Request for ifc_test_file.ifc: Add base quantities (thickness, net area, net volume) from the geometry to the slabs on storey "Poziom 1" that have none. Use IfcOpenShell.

First a look at what the model holds.

```python
import ifcopenshell
import ifcopenshell.util.element
import ifcopenshell.util.unit

model = ifcopenshell.open("ifc_test_file.ifc")
print(model.schema)
for unit_type in ("LENGTHUNIT", "AREAUNIT", "VOLUMEUNIT"):
    print(unit_type, ifcopenshell.util.unit.calculate_unit_scale(model, unit_type))
storey = next(s for s in model.by_type("IfcBuildingStorey") if s.Name == "Poziom 1")
slabs = [e for e in ifcopenshell.util.element.get_decomposition(storey) if e.is_a("IfcSlab")]
for e in sorted(slabs, key=lambda e: e.id()):
    print(e.id(), e.is_a(), e.Name, list(ifcopenshell.util.element.get_psets(e, qtos_only=True)), sep=" | ")
```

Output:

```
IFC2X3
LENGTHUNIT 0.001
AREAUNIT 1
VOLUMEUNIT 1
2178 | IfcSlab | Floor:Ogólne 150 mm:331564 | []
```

```python
import ifcopenshell
import ifcopenshell.api.pset
import ifcopenshell.geom
import ifcopenshell.util.element
import ifcopenshell.util.shape
import ifcopenshell.util.unit

model = ifcopenshell.open("ifc_test_file.ifc")
unit_scale = ifcopenshell.util.unit.calculate_unit_scale(model)
area_scale = ifcopenshell.util.unit.calculate_unit_scale(model, "AREAUNIT")
volume_scale = ifcopenshell.util.unit.calculate_unit_scale(model, "VOLUMEUNIT")
settings = ifcopenshell.geom.settings()

storey = next(s for s in model.by_type("IfcBuildingStorey") if s.Name == "Poziom 1")
slabs = [e for e in ifcopenshell.util.element.get_decomposition(storey) if e.is_a("IfcSlab")]

for e in sorted(slabs, key=lambda e: e.id()):
    if ifcopenshell.util.element.get_psets(e, qtos_only=True, should_inherit=False):
        continue
    # Geometry comes back in metres, in the element's own axes.
    shape = ifcopenshell.geom.create_shape(settings, e)
    values = {
        "Width": ifcopenshell.util.shape.get_z(shape.geometry) / unit_scale,
        "NetArea": ifcopenshell.util.shape.get_footprint_area(shape.geometry) / area_scale,
        "NetVolume": ifcopenshell.util.shape.get_volume(shape.geometry) / volume_scale,
    }
    qto = ifcopenshell.api.pset.add_qto(model, product=e, name="BaseQuantities")
    ifcopenshell.api.pset.edit_qto(model, qto=qto, properties=values)
    print(e.id(), {k: round(v, 3) for k, v in values.items()})

model.write("ifc_test_file_rev.ifc")
```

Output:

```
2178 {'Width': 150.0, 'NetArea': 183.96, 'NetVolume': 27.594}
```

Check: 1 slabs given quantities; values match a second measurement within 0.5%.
